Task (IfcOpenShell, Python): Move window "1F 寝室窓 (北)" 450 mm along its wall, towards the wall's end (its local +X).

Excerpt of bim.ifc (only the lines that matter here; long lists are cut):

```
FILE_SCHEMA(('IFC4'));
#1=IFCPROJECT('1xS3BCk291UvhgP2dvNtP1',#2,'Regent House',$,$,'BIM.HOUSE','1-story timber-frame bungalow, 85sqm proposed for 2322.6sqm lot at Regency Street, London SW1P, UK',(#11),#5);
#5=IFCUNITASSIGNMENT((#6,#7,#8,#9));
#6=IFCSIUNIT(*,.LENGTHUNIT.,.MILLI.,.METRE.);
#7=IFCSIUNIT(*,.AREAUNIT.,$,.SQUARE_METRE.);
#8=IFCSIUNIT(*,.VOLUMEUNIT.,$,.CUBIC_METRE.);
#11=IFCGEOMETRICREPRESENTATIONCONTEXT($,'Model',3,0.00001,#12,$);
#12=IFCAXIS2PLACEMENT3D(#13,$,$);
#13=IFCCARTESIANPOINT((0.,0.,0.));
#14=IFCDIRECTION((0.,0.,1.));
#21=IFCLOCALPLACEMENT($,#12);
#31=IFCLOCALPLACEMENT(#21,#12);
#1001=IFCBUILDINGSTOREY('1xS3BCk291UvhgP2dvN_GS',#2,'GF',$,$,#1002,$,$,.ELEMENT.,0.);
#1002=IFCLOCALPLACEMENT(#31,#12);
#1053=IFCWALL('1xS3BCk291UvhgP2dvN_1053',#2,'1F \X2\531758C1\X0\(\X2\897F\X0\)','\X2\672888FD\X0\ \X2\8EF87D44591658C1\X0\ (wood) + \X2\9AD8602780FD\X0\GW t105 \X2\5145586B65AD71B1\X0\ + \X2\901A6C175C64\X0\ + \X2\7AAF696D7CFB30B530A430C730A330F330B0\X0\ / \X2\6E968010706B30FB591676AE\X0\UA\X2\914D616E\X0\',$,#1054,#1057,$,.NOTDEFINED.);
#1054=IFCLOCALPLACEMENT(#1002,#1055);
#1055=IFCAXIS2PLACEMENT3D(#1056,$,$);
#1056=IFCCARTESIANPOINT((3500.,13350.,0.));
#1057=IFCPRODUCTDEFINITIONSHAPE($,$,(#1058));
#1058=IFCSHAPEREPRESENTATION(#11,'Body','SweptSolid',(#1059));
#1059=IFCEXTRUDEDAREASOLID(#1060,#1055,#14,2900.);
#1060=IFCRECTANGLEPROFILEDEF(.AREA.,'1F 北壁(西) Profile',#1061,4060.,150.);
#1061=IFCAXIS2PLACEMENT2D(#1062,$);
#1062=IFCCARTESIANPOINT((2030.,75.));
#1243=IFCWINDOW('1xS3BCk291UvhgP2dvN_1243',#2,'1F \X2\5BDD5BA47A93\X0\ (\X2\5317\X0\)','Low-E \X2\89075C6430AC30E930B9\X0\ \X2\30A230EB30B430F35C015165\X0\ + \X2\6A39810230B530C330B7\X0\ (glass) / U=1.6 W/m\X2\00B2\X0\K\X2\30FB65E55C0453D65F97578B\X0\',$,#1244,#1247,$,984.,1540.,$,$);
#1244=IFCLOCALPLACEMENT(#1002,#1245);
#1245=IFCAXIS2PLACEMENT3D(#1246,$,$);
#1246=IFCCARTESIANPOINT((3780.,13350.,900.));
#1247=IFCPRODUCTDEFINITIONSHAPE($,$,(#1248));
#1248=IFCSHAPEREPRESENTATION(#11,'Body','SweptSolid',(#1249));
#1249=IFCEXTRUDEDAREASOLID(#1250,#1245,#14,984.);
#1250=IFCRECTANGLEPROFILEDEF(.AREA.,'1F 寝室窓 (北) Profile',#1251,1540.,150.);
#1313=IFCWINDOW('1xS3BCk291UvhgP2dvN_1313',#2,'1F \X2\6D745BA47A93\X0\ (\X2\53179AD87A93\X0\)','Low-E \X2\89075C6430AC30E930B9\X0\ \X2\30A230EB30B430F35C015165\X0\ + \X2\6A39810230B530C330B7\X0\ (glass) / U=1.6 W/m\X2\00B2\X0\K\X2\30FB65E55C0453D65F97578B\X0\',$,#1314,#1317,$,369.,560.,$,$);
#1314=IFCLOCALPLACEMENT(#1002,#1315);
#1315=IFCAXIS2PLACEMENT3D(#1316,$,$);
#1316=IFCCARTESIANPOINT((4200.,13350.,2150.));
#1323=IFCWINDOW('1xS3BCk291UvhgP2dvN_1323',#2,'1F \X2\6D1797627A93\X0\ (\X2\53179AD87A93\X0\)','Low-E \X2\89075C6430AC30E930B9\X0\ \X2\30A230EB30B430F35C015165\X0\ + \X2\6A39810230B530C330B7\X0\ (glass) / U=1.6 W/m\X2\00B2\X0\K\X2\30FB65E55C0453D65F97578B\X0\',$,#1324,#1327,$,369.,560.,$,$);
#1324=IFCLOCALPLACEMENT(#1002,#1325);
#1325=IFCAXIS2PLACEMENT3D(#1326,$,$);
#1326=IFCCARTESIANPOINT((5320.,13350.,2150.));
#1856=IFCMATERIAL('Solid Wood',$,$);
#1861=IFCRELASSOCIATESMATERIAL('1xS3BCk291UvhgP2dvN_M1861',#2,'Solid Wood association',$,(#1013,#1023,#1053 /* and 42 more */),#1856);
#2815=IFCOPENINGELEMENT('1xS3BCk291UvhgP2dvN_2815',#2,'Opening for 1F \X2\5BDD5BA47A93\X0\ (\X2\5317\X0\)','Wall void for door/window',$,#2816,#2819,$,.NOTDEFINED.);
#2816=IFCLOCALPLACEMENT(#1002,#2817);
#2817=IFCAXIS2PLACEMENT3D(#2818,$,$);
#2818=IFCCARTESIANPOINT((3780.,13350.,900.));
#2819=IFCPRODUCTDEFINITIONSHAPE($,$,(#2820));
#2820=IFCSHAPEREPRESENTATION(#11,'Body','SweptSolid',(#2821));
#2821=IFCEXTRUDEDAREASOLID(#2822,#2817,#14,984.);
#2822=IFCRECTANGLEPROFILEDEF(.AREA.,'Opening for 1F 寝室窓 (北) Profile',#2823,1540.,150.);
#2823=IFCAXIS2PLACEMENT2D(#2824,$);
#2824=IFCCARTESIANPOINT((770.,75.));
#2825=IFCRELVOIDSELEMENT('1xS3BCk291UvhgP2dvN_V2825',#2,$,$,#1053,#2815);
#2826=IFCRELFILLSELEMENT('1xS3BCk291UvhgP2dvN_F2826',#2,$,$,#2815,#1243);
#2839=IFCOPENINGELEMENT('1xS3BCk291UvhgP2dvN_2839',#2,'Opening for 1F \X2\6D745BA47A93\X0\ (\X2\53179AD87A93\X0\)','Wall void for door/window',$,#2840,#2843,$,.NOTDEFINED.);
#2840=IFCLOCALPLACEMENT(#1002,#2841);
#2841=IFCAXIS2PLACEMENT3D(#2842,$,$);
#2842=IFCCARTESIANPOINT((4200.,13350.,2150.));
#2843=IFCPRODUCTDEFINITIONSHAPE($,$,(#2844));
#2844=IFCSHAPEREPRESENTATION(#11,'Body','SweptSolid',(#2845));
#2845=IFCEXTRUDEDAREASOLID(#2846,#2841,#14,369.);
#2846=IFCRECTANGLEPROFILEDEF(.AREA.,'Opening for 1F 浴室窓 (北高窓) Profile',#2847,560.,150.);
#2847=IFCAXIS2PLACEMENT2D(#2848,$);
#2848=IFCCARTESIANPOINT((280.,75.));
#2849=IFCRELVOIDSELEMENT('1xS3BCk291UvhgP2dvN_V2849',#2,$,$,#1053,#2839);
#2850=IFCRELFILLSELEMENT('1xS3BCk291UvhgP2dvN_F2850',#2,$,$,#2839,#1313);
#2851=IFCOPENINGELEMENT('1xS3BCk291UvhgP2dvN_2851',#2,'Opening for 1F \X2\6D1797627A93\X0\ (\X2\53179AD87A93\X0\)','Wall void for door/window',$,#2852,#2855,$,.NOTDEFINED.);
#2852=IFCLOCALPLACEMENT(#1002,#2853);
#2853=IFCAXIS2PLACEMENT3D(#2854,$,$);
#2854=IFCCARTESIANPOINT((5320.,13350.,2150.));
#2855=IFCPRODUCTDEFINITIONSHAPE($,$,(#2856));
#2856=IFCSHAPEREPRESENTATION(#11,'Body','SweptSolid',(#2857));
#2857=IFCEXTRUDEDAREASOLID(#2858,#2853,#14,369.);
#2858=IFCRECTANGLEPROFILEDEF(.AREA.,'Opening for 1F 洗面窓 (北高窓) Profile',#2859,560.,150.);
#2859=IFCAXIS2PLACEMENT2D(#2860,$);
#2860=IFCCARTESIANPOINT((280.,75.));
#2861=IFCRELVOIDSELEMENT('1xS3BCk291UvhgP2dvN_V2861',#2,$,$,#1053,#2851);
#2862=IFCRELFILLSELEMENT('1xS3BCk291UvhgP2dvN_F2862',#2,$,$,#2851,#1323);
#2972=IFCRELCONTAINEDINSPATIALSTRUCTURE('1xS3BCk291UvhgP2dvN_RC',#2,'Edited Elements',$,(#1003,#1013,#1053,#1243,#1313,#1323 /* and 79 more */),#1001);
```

```python
import ifcopenshell
import ifcopenshell.api.geometry
import ifcopenshell.util.placement

model = ifcopenshell.open("bim.ifc")

window = model.by_id(1243)
opening = window.FillsVoids[0].RelatingOpeningElement
wall = opening.VoidsElements[0].RelatingBuildingElement

wall_matrix = ifcopenshell.util.placement.get_local_placement(wall.ObjectPlacement)
shift = wall_matrix[:3, 0] * 450.0
before = ifcopenshell.util.placement.get_local_placement(window.ObjectPlacement)[:3, 3].copy()

# The window is not placed relative to its opening, so move both.
for product in (opening, window):
    matrix = ifcopenshell.util.placement.get_local_placement(product.ObjectPlacement)
    matrix[:3, 3] += shift
    ifcopenshell.api.geometry.edit_object_placement(model, product=product, matrix=matrix, is_si=False)

after = ifcopenshell.util.placement.get_local_placement(window.ObjectPlacement)[:3, 3]
print("window moved by", (after - before).round(3) + 0.0)

model.write("bim_rev.ifc")
```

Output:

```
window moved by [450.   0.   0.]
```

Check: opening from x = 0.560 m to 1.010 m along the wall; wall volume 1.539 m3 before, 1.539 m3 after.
